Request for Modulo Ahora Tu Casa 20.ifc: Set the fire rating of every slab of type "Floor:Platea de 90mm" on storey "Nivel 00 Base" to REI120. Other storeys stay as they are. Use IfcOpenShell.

First a look at what the model holds.

```python
import ifcopenshell
import ifcopenshell.util.element

model = ifcopenshell.open("Modulo Ahora Tu Casa 20.ifc")
print(model.schema)
storey = next(s for s in model.by_type("IfcBuildingStorey") if s.Name == "Nivel 00 Base")
slabs = [e for e in ifcopenshell.util.element.get_decomposition(storey) if e.is_a("IfcSlab")]
seen = {}
for e in slabs:
    element_type = ifcopenshell.util.element.get_type(e)
    key = (element_type.Name if element_type != e and element_type else None, ifcopenshell.util.element.get_pset(e, "Pset_SlabCommon", "FireRating"))
    seen[key] = seen.get(key, 0) + 1
for (name, value), count in sorted(seen.items(), key=str):
    print(count, "x", name, "|", value)
```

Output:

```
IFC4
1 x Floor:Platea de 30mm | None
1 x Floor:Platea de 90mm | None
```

```python
import ifcopenshell
import ifcopenshell.api.pset
import ifcopenshell.util.element

model = ifcopenshell.open("Modulo Ahora Tu Casa 20.ifc")

storey = next(s for s in model.by_type("IfcBuildingStorey") if s.Name == "Nivel 00 Base")
slabs = [e for e in ifcopenshell.util.element.get_decomposition(storey) if e.is_a("IfcSlab")]

count = 0
for e in slabs:
    element_type = ifcopenshell.util.element.get_type(e)
    if element_type in (None, e) or element_type.Name != "Floor:Platea de 90mm":
        continue
    # add_pset returns the element's existing set when there is one.
    pset = ifcopenshell.api.pset.add_pset(model, product=e, name="Pset_SlabCommon")
    ifcopenshell.api.pset.edit_pset(model, pset=pset, properties={"FireRating": "REI120"})
    count += 1

print(count, "slabs updated")

model.write("Modulo Ahora Tu Casa 20-out.ifc")
```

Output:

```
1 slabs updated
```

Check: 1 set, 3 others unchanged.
